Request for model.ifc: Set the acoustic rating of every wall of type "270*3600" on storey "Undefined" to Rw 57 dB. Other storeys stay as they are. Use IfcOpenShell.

First a look at what the model holds.

```python
import ifcopenshell
import ifcopenshell.util.element

model = ifcopenshell.open("model.ifc")
print(model.schema)
storey = next(s for s in model.by_type("IfcBuildingStorey") if s.Name == "Undefined")
walls = [e for e in ifcopenshell.util.element.get_decomposition(storey) if e.is_a("IfcWall")]
seen = {}
for e in walls:
    element_type = ifcopenshell.util.element.get_type(e)
    key = (element_type.Name if element_type != e and element_type else None, ifcopenshell.util.element.get_pset(e, "Pset_WallCommon", "AcousticRating"))
    seen[key] = seen.get(key, 0) + 1
for (name, value), count in sorted(seen.items(), key=str):
    print(count, "x", name, "|", value)
```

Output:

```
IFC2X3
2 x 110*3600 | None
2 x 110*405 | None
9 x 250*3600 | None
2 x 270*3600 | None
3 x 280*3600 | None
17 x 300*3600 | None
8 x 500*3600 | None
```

```python
import ifcopenshell
import ifcopenshell.api.pset
import ifcopenshell.util.element

model = ifcopenshell.open("model.ifc")

storey = next(s for s in model.by_type("IfcBuildingStorey") if s.Name == "Undefined")
walls = [e for e in ifcopenshell.util.element.get_decomposition(storey) if e.is_a("IfcWall")]

count = 0
for e in walls:
    element_type = ifcopenshell.util.element.get_type(e)
    if element_type in (None, e) or element_type.Name != "270*3600":
        continue
    found = ifcopenshell.util.element.get_pset(e, "Pset_WallCommon", should_inherit=False)
    if found:
        pset = model.by_id(found["id"])
        if len(ifcopenshell.util.element.get_elements_by_pset(pset)) > 1:
            pset = ifcopenshell.api.pset.unshare_pset(model, products=[e], pset=pset)[0]
    else:
        pset = ifcopenshell.api.pset.add_pset(model, product=e, name="Pset_WallCommon")
    ifcopenshell.api.pset.edit_pset(model, pset=pset, properties={"AcousticRating": "Rw 57 dB"})
    count += 1

print(count, "walls updated")

model.write("model_v2.ifc")
```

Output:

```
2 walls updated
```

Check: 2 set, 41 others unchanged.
